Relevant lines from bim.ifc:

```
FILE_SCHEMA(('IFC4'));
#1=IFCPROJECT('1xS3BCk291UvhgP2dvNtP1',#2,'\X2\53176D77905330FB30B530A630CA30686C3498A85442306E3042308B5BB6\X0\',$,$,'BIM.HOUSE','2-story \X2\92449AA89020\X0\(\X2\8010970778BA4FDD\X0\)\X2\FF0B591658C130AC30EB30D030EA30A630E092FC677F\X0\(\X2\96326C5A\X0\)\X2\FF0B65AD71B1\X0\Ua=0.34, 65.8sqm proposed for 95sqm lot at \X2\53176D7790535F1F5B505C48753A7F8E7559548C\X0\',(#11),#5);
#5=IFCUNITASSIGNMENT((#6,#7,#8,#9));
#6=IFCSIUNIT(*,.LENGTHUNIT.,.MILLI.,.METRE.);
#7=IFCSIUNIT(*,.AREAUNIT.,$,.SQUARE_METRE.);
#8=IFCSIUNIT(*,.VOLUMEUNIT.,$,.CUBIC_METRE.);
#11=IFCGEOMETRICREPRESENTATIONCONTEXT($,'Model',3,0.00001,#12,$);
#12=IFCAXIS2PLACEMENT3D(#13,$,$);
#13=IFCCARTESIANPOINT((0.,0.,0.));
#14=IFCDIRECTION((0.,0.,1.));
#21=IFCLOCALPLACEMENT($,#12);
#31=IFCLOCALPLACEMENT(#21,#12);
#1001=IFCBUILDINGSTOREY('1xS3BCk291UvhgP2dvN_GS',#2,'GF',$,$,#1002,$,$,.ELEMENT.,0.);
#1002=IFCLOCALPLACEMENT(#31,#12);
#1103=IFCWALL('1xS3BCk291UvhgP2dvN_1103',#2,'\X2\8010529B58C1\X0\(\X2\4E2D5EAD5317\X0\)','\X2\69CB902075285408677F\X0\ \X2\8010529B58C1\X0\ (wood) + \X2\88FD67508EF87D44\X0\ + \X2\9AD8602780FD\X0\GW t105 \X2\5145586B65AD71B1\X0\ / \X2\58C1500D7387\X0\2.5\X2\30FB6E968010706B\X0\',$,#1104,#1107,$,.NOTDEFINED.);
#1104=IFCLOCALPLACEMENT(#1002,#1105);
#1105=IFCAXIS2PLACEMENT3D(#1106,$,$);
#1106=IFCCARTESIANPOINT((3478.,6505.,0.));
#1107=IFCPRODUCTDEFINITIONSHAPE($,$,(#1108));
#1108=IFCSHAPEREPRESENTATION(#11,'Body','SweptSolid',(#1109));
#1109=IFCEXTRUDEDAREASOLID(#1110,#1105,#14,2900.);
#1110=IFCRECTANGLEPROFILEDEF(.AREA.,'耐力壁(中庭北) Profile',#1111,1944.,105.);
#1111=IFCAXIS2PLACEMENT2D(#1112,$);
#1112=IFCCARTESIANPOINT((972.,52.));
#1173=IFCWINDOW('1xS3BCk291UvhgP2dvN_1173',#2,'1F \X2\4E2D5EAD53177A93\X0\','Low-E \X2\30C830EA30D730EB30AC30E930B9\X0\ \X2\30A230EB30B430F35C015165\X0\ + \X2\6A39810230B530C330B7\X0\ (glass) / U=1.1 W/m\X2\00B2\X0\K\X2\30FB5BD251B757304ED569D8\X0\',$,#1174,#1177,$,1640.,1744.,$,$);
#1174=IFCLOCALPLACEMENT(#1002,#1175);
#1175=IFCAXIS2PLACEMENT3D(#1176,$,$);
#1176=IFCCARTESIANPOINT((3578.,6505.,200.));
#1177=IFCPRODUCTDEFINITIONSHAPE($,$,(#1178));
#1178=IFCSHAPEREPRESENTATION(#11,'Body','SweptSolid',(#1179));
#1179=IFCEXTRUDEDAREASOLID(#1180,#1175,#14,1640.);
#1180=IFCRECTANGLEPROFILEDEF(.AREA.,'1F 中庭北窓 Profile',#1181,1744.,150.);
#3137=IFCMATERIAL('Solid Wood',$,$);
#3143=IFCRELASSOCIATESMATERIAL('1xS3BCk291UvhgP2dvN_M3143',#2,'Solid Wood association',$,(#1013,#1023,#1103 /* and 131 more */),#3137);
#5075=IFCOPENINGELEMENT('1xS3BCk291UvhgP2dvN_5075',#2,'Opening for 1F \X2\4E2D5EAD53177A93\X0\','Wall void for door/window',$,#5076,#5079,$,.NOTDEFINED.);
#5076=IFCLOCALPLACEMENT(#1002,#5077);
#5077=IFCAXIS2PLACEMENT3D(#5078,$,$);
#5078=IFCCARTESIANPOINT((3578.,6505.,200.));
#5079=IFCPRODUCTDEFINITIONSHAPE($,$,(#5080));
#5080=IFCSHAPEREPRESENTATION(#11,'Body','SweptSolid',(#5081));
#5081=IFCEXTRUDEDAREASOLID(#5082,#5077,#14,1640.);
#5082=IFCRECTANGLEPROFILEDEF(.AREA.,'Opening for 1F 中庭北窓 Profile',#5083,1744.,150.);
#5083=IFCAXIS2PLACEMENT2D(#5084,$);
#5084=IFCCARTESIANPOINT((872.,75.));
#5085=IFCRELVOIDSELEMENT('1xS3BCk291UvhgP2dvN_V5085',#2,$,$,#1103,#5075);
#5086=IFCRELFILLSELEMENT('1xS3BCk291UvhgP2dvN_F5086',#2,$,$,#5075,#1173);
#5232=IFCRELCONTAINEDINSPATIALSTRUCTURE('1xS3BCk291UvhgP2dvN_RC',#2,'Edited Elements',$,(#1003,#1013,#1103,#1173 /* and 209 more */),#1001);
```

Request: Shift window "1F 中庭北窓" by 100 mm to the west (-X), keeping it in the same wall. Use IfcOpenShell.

```python
import ifcopenshell
import ifcopenshell.api.geometry
import ifcopenshell.util.placement

model = ifcopenshell.open("bim.ifc")

window = model.by_guid("1xS3BCk291UvhgP2dvN_1173")
opening = window.FillsVoids[0].RelatingOpeningElement
wall = opening.VoidsElements[0].RelatingBuildingElement

wall_matrix = ifcopenshell.util.placement.get_local_placement(wall.ObjectPlacement)
shift = wall_matrix[:3, 0] * -100.0
before = ifcopenshell.util.placement.get_local_placement(window.ObjectPlacement)[:3, 3].copy()

# The window is not placed relative to its opening, so move both.
for product in (opening, window):
    matrix = ifcopenshell.util.placement.get_local_placement(product.ObjectPlacement)
    matrix[:3, 3] += shift
    ifcopenshell.api.geometry.edit_object_placement(model, product=product, matrix=matrix, is_si=False)

after = ifcopenshell.util.placement.get_local_placement(window.ObjectPlacement)[:3, 3]
print("window moved by", (after - before).round(3) + 0.0)

model.write("bim_updated.ifc")
```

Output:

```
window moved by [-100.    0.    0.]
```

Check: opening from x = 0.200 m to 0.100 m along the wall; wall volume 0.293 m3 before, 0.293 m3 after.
